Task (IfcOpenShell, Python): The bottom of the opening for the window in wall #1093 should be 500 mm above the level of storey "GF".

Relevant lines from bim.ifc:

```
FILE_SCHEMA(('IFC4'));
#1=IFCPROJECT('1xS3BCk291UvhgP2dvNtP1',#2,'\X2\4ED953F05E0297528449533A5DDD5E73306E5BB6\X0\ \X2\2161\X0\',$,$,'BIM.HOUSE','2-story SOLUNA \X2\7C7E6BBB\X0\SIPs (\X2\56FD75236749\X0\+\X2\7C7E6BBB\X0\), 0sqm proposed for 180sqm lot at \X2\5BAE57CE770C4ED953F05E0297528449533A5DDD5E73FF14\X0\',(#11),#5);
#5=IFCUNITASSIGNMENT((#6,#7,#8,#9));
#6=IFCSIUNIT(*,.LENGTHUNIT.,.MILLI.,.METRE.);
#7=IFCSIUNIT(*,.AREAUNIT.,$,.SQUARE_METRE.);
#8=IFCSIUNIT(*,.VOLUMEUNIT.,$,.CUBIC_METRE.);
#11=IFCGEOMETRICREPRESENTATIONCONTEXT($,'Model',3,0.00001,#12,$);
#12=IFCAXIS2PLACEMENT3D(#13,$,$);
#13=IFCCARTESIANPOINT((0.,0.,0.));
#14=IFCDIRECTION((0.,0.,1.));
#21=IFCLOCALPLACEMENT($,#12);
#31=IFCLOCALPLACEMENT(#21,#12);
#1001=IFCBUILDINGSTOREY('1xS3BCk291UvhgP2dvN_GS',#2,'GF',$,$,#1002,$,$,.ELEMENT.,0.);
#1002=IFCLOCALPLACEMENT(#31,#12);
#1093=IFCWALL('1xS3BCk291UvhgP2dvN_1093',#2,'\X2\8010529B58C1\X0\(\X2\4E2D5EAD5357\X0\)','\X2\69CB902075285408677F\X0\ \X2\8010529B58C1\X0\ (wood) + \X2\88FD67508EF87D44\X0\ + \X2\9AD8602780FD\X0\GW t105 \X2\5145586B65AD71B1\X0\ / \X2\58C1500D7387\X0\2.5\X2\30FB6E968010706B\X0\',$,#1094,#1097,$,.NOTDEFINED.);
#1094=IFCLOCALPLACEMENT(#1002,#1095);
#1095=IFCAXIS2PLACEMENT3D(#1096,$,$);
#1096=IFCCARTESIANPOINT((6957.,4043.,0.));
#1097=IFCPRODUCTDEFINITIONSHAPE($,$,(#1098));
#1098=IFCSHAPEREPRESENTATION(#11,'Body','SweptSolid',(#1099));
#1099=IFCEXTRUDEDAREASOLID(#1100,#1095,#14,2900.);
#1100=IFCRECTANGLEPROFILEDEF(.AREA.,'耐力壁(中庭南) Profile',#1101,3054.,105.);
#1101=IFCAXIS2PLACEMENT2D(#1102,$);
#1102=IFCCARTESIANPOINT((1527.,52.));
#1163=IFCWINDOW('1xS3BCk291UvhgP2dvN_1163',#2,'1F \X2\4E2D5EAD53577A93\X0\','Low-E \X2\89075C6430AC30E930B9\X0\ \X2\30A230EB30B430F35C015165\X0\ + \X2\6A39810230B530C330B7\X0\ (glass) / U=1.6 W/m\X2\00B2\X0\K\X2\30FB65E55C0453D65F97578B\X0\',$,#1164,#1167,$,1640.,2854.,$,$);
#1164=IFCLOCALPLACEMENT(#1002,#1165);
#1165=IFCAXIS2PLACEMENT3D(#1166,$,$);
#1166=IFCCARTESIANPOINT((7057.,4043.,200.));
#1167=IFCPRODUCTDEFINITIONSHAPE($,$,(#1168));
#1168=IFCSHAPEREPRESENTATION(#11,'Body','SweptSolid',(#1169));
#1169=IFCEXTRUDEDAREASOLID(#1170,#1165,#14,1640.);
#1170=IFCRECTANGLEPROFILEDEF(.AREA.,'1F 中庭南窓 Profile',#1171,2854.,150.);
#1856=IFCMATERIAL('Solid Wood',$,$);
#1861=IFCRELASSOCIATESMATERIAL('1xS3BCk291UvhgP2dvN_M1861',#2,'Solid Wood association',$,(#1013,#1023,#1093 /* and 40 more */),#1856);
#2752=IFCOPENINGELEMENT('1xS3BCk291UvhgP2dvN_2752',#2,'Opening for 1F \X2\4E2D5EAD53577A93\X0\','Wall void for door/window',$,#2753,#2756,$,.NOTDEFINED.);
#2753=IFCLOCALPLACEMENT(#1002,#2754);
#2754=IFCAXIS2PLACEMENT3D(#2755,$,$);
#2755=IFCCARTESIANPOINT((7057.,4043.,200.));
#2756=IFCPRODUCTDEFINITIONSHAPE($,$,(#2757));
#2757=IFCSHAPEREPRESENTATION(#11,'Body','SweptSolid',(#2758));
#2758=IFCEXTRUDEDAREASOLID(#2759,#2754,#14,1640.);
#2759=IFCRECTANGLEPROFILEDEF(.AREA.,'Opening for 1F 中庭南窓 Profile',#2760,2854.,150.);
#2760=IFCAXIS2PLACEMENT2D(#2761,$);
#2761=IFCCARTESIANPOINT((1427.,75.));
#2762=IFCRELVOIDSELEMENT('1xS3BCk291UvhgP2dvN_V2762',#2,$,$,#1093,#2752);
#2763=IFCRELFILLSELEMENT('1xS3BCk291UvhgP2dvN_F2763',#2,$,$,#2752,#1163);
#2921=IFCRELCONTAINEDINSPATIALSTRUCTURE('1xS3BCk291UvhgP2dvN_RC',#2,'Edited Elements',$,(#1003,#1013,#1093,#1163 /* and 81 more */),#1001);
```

```python
import numpy as np
import ifcopenshell
import ifcopenshell.api.geometry
import ifcopenshell.geom
import ifcopenshell.util.element
import ifcopenshell.util.placement
import ifcopenshell.util.shape
import ifcopenshell.util.unit

model = ifcopenshell.open("bim.ifc")
unit_scale = ifcopenshell.util.unit.calculate_unit_scale(model)

window = model.by_guid("1xS3BCk291UvhgP2dvN_1163")
opening = window.FillsVoids[0].RelatingOpeningElement
storey = ifcopenshell.util.element.get_container(window, ifc_class="IfcBuildingStorey")
level = ifcopenshell.util.placement.get_local_placement(storey.ObjectPlacement)[2, 3]

# The opening's origin need not be at the sill, so measure its lowest point.
shape = ifcopenshell.geom.create_shape(ifcopenshell.geom.settings(), opening)
bottom = ifcopenshell.util.shape.get_shape_bottom_elevation(shape, shape.geometry) / unit_scale
dz = level + 0.5 / unit_scale - bottom

shift = np.array([0.0, 0.0, dz])
# The window is not placed relative to its opening, so move both.
for product in (opening, window):
    matrix = ifcopenshell.util.placement.get_local_placement(product.ObjectPlacement)
    matrix[:3, 3] += shift
    ifcopenshell.api.geometry.edit_object_placement(model, product=product, matrix=matrix, is_si=False)

print(f"moved by {dz * unit_scale:+.3f} m")

model.write("bim-out.ifc")
```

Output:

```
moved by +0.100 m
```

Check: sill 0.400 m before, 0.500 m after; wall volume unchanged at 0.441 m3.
